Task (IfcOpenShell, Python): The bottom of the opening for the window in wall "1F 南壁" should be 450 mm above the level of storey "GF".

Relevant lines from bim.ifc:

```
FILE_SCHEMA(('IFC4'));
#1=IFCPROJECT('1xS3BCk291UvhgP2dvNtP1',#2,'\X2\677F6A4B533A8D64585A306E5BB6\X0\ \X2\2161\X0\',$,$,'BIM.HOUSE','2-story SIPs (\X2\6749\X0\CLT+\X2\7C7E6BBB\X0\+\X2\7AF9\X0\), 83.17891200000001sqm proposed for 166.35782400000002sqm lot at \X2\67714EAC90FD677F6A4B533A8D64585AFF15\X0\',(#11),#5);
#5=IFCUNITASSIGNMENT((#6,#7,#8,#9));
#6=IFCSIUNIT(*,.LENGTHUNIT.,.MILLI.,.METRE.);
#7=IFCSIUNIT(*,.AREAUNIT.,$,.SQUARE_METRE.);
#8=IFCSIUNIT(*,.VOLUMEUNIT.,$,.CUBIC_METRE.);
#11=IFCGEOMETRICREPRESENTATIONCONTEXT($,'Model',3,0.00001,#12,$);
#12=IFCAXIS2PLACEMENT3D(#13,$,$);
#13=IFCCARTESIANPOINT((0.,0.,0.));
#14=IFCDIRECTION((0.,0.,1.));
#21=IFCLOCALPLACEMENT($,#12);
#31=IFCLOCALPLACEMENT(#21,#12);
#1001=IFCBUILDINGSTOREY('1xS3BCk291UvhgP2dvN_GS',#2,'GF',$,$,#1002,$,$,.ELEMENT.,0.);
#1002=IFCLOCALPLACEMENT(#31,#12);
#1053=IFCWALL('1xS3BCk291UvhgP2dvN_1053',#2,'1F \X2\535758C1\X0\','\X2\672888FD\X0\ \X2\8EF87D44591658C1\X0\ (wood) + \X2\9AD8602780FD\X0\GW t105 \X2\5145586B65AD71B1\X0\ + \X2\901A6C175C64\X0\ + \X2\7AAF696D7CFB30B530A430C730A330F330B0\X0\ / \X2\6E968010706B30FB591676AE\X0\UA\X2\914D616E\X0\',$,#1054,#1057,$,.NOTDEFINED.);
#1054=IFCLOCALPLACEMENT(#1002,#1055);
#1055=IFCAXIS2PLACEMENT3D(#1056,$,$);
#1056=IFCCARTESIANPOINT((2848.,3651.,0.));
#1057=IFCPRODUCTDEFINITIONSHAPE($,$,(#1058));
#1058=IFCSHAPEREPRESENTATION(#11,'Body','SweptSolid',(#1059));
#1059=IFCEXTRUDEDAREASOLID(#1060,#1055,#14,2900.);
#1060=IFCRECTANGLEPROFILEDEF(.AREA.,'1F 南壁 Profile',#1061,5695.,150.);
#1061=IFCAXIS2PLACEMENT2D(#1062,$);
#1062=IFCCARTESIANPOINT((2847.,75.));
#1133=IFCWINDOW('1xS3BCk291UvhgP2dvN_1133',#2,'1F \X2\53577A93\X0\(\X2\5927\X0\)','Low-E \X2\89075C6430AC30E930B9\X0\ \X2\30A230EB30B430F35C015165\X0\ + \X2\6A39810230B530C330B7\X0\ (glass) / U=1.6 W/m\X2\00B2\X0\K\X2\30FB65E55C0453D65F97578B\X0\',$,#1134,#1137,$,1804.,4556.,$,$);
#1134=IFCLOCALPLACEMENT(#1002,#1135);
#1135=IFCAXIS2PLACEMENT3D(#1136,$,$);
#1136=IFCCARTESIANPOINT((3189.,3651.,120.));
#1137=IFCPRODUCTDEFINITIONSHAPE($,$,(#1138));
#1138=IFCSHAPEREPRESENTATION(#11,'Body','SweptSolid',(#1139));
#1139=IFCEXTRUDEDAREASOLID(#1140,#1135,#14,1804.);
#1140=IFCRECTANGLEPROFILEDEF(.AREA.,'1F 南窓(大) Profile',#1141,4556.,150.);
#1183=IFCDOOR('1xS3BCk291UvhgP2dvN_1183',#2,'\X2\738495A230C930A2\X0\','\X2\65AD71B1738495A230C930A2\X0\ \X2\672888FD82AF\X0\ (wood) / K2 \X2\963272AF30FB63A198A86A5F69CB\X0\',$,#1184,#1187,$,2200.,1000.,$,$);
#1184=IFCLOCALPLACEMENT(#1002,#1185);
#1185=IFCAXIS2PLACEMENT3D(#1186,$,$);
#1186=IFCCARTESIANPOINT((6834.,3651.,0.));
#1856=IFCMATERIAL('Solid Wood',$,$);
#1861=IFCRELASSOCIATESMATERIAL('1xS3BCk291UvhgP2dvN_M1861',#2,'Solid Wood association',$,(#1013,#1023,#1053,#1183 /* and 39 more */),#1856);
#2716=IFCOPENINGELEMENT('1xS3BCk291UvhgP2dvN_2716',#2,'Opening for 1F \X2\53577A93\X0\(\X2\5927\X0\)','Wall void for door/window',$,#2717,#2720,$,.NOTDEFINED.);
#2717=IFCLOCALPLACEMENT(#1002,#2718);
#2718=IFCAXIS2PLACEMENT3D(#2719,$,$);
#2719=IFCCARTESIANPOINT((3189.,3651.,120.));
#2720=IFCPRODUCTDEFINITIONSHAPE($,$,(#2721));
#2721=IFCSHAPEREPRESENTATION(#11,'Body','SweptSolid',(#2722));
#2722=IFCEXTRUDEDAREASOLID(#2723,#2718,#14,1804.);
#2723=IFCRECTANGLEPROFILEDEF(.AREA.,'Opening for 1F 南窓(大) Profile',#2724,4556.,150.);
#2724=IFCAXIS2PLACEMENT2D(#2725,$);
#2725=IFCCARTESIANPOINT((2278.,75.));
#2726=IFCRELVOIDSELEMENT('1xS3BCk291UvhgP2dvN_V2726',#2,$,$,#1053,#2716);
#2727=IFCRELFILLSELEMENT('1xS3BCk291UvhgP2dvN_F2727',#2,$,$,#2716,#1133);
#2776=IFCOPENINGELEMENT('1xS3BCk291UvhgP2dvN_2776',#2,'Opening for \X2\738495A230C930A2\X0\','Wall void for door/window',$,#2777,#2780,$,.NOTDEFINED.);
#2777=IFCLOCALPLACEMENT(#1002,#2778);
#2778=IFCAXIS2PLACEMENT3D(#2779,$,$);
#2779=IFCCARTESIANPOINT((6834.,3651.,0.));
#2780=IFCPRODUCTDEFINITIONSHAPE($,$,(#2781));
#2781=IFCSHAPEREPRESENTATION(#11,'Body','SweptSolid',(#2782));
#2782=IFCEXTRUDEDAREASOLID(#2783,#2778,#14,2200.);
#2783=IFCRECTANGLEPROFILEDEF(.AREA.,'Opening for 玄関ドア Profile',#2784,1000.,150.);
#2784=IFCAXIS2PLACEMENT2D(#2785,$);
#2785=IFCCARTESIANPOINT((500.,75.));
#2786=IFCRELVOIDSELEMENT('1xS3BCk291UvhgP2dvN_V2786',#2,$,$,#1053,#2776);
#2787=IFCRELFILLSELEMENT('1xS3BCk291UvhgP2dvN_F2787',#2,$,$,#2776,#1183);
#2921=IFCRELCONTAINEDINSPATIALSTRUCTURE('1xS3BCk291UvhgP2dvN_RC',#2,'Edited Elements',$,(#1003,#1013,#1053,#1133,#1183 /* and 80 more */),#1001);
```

```python
import numpy as np
import ifcopenshell
import ifcopenshell.api.geometry
import ifcopenshell.geom
import ifcopenshell.util.element
import ifcopenshell.util.placement
import ifcopenshell.util.shape
import ifcopenshell.util.unit

model = ifcopenshell.open("bim.ifc")
unit_scale = ifcopenshell.util.unit.calculate_unit_scale(model)

window = model.by_guid("1xS3BCk291UvhgP2dvN_1133")
opening = window.FillsVoids[0].RelatingOpeningElement
storey = ifcopenshell.util.element.get_container(window, ifc_class="IfcBuildingStorey")
level = ifcopenshell.util.placement.get_local_placement(storey.ObjectPlacement)[2, 3]

# The opening's origin need not be at the sill, so measure its lowest point.
shape = ifcopenshell.geom.create_shape(ifcopenshell.geom.settings(), opening)
bottom = ifcopenshell.util.shape.get_shape_bottom_elevation(shape, shape.geometry) / unit_scale
dz = level + 0.45 / unit_scale - bottom

shift = np.array([0.0, 0.0, dz])
# The window is not placed relative to its opening, so move both.
for product in (opening, window):
    matrix = ifcopenshell.util.placement.get_local_placement(product.ObjectPlacement)
    matrix[:3, 3] += shift
    ifcopenshell.api.geometry.edit_object_placement(model, product=product, matrix=matrix, is_si=False)

print(f"moved by {dz * unit_scale:+.3f} m")

model.write("bim_rev.ifc")
```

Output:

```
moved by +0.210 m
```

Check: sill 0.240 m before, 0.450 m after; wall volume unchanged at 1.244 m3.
